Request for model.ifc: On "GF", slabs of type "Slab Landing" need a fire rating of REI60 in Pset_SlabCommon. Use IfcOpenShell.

First a look at what the model holds.

```python
import ifcopenshell
import ifcopenshell.util.element

model = ifcopenshell.open("model.ifc")
print(model.schema)
storey = next(s for s in model.by_type("IfcBuildingStorey") if s.Name == "GF")
slabs = [e for e in ifcopenshell.util.element.get_decomposition(storey) if e.is_a("IfcSlab")]
seen = {}
for e in slabs:
    element_type = ifcopenshell.util.element.get_type(e)
    key = (element_type.Name if element_type != e and element_type else None, ifcopenshell.util.element.get_pset(e, "Pset_SlabCommon", "FireRating"))
    seen[key] = seen.get(key, 0) + 1
for (name, value), count in sorted(seen.items(), key=str):
    print(count, "x", name, "|", value)
```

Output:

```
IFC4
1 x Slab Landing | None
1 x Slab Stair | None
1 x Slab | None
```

```python
import ifcopenshell
import ifcopenshell.api.pset
import ifcopenshell.util.element

model = ifcopenshell.open("model.ifc")

storey = next(s for s in model.by_type("IfcBuildingStorey") if s.Name == "GF")
slabs = [e for e in ifcopenshell.util.element.get_decomposition(storey) if e.is_a("IfcSlab")]

count = 0
for e in slabs:
    element_type = ifcopenshell.util.element.get_type(e)
    if element_type in (None, e) or element_type.Name != "Slab Landing":
        continue
    # add_pset returns the element's existing set when there is one.
    pset = ifcopenshell.api.pset.add_pset(model, product=e, name="Pset_SlabCommon")
    ifcopenshell.api.pset.edit_pset(model, pset=pset, properties={"FireRating": "REI60"})
    count += 1

print(count, "slabs updated")

model.write("model-out.ifc")
```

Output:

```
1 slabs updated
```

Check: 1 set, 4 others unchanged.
